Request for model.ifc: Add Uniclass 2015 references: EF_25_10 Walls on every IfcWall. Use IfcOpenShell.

First a look at what the model holds.

```python
import ifcopenshell

model = ifcopenshell.open("model.ifc")
print(model.schema)
print("classifications:", [c.Name for c in model.by_type("IfcClassification")])
for ifc_class in ("IfcDoor", "IfcRoof", "IfcStair", "IfcWall", "IfcWindow"):
    print(ifc_class, len(model.by_type(ifc_class)))
```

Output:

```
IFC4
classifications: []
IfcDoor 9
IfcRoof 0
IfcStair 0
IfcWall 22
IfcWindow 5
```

```python
import ifcopenshell
import ifcopenshell.api.classification

model = ifcopenshell.open("model.ifc")

system = ifcopenshell.api.classification.add_classification(model, classification="Uniclass 2015")

codes = {
    "IfcWall": ("EF_25_10", "Walls"),
}
for ifc_class, (code, name) in codes.items():
    products = model.by_type(ifc_class)
    ifcopenshell.api.classification.add_reference(
        model, products=products, classification=system, identification=code, name=name
    )
    print(code, len(products))

model.write("model-out.ifc")
```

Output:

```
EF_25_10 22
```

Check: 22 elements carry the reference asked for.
